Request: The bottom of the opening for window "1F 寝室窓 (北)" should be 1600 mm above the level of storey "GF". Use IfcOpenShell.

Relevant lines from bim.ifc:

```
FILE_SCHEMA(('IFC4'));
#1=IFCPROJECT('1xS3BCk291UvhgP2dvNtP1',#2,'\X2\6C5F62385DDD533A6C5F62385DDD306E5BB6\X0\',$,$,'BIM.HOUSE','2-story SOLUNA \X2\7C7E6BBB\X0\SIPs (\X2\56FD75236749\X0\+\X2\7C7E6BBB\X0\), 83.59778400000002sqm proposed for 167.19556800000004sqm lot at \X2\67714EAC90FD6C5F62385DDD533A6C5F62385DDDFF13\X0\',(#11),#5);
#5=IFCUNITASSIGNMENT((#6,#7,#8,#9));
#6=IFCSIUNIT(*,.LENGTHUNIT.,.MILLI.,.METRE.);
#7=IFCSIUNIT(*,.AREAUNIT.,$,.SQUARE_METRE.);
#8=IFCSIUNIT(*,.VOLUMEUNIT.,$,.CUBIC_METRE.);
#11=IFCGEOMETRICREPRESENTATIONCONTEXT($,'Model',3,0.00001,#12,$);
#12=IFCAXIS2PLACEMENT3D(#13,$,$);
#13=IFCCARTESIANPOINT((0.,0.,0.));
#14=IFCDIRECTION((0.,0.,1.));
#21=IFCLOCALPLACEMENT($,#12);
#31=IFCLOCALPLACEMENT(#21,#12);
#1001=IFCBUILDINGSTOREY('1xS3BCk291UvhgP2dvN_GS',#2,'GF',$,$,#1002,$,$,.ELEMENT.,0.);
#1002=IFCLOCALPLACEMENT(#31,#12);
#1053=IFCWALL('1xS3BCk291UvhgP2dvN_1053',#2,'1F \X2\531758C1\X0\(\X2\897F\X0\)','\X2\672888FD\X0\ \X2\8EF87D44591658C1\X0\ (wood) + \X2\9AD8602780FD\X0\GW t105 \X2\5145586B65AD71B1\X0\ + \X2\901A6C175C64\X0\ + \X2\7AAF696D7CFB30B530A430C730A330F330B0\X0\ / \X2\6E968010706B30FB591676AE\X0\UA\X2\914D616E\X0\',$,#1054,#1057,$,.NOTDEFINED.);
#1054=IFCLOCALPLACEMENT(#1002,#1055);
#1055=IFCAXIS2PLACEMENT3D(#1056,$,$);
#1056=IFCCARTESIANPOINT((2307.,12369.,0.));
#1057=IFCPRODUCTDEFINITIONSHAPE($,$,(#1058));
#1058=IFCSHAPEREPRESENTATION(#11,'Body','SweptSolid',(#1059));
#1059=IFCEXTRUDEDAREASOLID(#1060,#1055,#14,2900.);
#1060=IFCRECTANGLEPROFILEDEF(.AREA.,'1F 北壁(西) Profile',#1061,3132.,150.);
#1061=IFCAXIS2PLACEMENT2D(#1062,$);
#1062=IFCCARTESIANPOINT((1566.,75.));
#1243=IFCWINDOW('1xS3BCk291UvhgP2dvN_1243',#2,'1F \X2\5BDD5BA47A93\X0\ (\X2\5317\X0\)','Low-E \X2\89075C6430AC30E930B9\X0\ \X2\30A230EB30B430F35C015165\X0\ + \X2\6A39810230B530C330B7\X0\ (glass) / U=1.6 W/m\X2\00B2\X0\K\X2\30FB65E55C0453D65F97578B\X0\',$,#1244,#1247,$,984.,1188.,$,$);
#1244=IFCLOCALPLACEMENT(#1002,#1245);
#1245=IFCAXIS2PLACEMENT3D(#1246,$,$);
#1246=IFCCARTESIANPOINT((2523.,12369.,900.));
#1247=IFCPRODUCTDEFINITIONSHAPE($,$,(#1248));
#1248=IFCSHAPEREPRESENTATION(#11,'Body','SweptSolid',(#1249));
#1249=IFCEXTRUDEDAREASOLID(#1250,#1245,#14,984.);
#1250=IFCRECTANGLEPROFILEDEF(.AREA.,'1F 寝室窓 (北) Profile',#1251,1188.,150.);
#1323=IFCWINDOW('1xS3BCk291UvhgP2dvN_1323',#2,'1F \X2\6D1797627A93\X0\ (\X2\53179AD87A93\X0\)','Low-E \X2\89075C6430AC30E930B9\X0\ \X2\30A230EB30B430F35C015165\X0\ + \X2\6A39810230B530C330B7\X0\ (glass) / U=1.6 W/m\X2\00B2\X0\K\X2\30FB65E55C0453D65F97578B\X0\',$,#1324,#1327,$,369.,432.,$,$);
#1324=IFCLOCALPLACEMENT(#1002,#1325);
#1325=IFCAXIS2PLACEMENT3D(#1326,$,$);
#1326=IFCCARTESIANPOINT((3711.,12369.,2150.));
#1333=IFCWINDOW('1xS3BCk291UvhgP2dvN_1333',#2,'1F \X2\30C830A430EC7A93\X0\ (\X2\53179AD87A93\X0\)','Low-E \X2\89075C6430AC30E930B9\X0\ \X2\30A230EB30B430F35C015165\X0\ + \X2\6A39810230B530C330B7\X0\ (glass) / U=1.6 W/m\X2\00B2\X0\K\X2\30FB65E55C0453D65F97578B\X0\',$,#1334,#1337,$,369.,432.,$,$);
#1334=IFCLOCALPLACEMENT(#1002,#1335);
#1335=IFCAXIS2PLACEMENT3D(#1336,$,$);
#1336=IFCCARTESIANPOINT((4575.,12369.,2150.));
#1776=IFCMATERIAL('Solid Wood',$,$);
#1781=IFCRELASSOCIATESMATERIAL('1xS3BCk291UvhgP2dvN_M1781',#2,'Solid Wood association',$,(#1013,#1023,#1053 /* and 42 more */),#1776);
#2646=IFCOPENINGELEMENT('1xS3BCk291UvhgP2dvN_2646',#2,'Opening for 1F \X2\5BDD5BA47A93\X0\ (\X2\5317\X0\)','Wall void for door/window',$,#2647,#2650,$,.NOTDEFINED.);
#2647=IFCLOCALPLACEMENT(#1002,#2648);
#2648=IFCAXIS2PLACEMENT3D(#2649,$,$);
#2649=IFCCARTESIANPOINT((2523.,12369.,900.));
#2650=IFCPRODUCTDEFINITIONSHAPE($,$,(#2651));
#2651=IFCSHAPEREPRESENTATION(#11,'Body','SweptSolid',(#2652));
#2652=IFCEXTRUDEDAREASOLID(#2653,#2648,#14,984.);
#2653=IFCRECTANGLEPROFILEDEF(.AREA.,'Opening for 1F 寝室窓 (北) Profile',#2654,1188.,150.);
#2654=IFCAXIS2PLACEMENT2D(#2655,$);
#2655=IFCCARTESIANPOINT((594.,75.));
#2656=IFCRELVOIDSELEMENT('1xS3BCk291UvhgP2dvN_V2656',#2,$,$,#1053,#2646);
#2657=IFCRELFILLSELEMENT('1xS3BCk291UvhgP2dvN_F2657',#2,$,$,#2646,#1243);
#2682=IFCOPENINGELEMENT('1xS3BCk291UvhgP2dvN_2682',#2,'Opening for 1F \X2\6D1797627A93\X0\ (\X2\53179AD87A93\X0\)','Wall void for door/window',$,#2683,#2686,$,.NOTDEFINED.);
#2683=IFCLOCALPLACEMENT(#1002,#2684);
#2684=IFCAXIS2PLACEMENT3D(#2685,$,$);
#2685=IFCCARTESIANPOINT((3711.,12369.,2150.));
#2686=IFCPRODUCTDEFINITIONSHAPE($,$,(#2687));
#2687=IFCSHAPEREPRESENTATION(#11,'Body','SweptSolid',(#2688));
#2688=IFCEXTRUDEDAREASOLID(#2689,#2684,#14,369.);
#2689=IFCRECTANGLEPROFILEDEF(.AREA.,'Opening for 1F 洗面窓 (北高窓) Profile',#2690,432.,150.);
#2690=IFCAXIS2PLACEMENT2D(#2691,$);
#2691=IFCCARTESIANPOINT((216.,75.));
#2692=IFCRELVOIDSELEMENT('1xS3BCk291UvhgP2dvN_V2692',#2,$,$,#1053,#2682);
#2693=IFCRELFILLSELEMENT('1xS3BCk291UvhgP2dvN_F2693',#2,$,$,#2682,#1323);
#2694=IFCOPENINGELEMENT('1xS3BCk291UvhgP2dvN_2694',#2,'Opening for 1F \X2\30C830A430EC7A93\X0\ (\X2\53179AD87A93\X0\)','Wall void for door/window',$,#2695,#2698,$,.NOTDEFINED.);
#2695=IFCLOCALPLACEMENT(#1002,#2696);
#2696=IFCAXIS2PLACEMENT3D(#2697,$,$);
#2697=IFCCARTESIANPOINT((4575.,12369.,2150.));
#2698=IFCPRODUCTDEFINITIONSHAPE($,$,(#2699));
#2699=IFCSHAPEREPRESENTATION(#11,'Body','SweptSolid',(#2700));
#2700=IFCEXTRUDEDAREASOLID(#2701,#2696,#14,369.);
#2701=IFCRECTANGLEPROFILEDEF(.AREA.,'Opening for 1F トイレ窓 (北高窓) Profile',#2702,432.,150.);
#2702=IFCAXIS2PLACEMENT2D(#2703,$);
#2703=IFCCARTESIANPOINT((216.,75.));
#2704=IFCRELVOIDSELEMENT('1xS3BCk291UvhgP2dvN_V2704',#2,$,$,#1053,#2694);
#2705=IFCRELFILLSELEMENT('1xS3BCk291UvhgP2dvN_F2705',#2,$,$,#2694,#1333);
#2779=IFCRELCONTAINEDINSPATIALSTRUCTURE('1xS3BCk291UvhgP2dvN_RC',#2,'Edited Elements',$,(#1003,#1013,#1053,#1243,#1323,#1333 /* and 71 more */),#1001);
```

```python
import numpy as np
import ifcopenshell
import ifcopenshell.api.geometry
import ifcopenshell.geom
import ifcopenshell.util.element
import ifcopenshell.util.placement
import ifcopenshell.util.shape
import ifcopenshell.util.unit

model = ifcopenshell.open("bim.ifc")
unit_scale = ifcopenshell.util.unit.calculate_unit_scale(model)

window = model.by_id(1243)
opening = window.FillsVoids[0].RelatingOpeningElement
storey = ifcopenshell.util.element.get_container(window, ifc_class="IfcBuildingStorey")
level = ifcopenshell.util.placement.get_local_placement(storey.ObjectPlacement)[2, 3]

# The opening's origin need not be at the sill, so measure its lowest point.
shape = ifcopenshell.geom.create_shape(ifcopenshell.geom.settings(), opening)
bottom = ifcopenshell.util.shape.get_shape_bottom_elevation(shape, shape.geometry) / unit_scale
dz = level + 1600.0 - bottom

shift = np.array([0.0, 0.0, dz])
# The window is not placed relative to its opening, so move both.
for product in (opening, window):
    matrix = ifcopenshell.util.placement.get_local_placement(product.ObjectPlacement)
    matrix[:3, 3] += shift
    ifcopenshell.api.geometry.edit_object_placement(model, product=product, matrix=matrix, is_si=False)

print(f"moved by {dz * unit_scale:+.3f} m")

model.write("bim-out.ifc")
```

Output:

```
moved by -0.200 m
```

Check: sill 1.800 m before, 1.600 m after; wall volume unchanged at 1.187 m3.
